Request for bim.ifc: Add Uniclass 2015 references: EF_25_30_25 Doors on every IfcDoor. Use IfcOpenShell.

First a look at what the model holds.

```python
import ifcopenshell

model = ifcopenshell.open("bim.ifc")
print(model.schema)
print("classifications:", [c.Name for c in model.by_type("IfcClassification")])
for ifc_class in ("IfcDoor", "IfcRoof", "IfcStair", "IfcWall", "IfcWindow"):
    print(ifc_class, len(model.by_type(ifc_class)))
```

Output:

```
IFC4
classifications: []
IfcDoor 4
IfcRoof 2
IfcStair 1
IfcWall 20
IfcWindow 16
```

```python
import ifcopenshell
import ifcopenshell.api.classification

model = ifcopenshell.open("bim.ifc")

system = ifcopenshell.api.classification.add_classification(model, classification="Uniclass 2015")

codes = {
    "IfcDoor": ("EF_25_30_25", "Doors"),
}
for ifc_class, (code, name) in codes.items():
    products = model.by_type(ifc_class)
    ifcopenshell.api.classification.add_reference(
        model, products=products, classification=system, identification=code, name=name
    )
    print(code, len(products))

model.write("bim_updated.ifc")
```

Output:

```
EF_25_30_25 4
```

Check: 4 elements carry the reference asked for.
